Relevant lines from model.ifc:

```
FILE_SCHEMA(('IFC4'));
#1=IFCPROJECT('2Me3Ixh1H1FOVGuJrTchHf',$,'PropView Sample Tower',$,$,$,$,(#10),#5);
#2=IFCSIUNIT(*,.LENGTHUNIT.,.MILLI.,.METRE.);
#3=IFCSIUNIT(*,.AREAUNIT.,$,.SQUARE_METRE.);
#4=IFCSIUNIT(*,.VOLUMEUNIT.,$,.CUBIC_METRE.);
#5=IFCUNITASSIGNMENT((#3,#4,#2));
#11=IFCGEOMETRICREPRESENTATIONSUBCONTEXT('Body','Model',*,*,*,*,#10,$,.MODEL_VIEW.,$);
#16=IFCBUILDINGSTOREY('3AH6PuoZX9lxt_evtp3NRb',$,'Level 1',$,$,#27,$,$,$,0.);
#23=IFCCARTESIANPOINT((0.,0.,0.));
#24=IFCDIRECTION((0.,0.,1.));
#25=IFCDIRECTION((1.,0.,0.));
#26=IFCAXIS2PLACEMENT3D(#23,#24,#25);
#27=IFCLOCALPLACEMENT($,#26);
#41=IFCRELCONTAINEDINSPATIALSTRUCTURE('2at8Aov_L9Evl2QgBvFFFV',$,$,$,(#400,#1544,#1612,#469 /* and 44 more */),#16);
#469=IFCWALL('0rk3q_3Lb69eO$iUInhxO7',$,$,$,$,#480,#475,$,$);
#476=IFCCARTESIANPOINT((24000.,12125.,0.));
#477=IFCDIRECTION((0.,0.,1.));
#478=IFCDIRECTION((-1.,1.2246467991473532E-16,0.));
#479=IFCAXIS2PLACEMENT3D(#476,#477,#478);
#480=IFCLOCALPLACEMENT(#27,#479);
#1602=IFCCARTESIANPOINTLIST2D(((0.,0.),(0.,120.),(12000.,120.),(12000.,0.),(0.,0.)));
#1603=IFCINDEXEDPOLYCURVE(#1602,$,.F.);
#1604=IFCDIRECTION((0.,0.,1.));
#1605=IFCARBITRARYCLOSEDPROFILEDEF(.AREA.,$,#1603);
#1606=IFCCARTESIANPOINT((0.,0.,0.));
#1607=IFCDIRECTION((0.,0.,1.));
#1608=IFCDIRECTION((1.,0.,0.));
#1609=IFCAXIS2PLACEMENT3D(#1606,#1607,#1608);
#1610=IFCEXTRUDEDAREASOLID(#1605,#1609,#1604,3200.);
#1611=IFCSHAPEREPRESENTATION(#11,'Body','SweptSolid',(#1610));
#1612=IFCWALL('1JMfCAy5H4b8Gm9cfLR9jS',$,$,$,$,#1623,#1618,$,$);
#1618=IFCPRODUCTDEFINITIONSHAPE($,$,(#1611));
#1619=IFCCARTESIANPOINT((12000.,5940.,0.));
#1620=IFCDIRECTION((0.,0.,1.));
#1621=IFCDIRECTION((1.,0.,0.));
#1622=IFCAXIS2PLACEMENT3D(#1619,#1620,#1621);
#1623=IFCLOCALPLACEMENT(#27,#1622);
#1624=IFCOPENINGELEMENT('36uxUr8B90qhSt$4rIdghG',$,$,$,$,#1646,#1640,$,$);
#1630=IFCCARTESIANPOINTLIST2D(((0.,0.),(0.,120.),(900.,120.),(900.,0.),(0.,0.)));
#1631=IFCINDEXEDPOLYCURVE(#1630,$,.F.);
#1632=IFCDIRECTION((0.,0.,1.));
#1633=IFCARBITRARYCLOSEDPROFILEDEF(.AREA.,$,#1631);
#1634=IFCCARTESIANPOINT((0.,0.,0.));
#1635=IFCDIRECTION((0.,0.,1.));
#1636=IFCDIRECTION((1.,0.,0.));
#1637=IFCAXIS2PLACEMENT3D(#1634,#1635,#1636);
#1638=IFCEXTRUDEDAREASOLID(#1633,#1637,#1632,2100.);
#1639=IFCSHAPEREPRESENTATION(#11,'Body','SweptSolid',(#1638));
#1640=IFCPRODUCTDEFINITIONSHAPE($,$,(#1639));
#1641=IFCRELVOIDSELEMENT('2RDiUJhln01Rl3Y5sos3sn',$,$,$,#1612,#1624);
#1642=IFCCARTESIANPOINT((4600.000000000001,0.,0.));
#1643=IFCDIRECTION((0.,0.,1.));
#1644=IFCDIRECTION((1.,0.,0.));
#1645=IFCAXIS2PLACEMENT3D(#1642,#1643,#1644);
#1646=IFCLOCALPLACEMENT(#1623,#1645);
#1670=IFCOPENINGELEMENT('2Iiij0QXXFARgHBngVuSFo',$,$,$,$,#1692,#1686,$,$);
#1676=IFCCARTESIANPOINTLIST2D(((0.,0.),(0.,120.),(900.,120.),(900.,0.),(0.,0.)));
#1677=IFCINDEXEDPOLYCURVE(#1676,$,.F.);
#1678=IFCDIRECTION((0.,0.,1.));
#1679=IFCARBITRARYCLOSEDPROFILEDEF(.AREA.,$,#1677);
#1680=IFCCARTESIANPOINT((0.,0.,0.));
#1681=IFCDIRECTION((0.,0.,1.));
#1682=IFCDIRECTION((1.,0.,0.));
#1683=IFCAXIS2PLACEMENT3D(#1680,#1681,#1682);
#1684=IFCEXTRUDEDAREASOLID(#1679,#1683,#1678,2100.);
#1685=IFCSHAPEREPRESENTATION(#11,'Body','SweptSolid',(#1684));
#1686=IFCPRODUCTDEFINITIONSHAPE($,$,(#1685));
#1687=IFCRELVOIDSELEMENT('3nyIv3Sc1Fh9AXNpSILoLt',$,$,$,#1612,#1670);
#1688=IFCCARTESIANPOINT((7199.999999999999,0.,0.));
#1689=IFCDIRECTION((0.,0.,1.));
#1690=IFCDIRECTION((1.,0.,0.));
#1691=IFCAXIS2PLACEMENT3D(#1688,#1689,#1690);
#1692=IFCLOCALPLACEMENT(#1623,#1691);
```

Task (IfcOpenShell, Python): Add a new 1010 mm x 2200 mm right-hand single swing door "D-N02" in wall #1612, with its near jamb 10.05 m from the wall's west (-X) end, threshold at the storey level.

```python
import numpy as np
import ifcopenshell
import ifcopenshell.api.feature
import ifcopenshell.api.geometry
import ifcopenshell.api.root
import ifcopenshell.api.spatial
import ifcopenshell.geom
import ifcopenshell.util.element
import ifcopenshell.util.placement
import ifcopenshell.util.representation
import ifcopenshell.util.shape
import ifcopenshell.util.unit

model = ifcopenshell.open("model.ifc")
unit_scale = ifcopenshell.util.unit.calculate_unit_scale(model)
settings = ifcopenshell.geom.settings()


def volume(element):
    """Net volume in cubic metres, openings subtracted."""
    shape = ifcopenshell.geom.create_shape(settings, element)
    return ifcopenshell.util.shape.get_volume(shape.geometry)


wall = model.by_guid("1JMfCAy5H4b8Gm9cfLR9jS")
storey = ifcopenshell.util.element.get_container(wall, ifc_class="IfcBuildingStorey")
context = ifcopenshell.util.representation.get_context(model, "Model", "Body", "MODEL_VIEW")
before = volume(wall)

width, height, from_end, sill = 1.01, 2.2, 10.05, 0.0  # metres

# The wall runs along its own X axis, and the end named is its -X end.
wall_shape = ifcopenshell.geom.create_shape(settings, wall)
x, y, z = ifcopenshell.util.shape.get_vertices(wall_shape.geometry).T
start = x.min() + from_end
face, thickness = float(y.min()), float(y.max() - y.min())
wall_matrix = ifcopenshell.util.placement.get_local_placement(wall.ObjectPlacement)
level = ifcopenshell.util.placement.get_local_placement(storey.ObjectPlacement)[2, 3]


def in_wall(x, y):
    """Placement at x, y metres in the wall's axes, at sill height."""
    matrix = wall_matrix.copy()
    matrix[:, 3] = wall_matrix @ np.array([x / unit_scale, y / unit_scale, 0.0, 1.0])
    matrix[2, 3] = level + sill / unit_scale
    return matrix


# Opening: a box that overshoots both wall faces by 50 mm.
opening = ifcopenshell.api.root.create_entity(model, ifc_class="IfcOpeningElement", predefined_type="OPENING")
box = ifcopenshell.api.geometry.add_wall_representation(
    model, context=context, length=width, height=height, thickness=thickness + 0.1
)
ifcopenshell.api.geometry.assign_representation(model, product=opening, representation=box)
ifcopenshell.api.geometry.edit_object_placement(model, product=opening, matrix=in_wall(start, face - 0.05), is_si=False)
ifcopenshell.api.feature.add_feature(model, feature=opening, element=wall)

door = ifcopenshell.api.root.create_entity(model, ifc_class="IfcDoor", name="D-N02", predefined_type="DOOR")
door.OverallWidth, door.OverallHeight = width / unit_scale, height / unit_scale
door.OperationType = "SINGLE_SWING_RIGHT"
body = ifcopenshell.api.geometry.add_door_representation(
    model,
    context=context,
    overall_width=door.OverallWidth,
    overall_height=door.OverallHeight,
    operation_type="SINGLE_SWING_RIGHT",
    lining_properties={"LiningDepth": thickness / unit_scale, "ThresholdDepth": thickness / unit_scale},
)
ifcopenshell.api.geometry.assign_representation(model, product=door, representation=body)
ifcopenshell.api.spatial.assign_container(model, products=[door], relating_structure=storey)
ifcopenshell.api.feature.add_filling(model, opening=opening, element=door)

# The lining spans the wall, so the door starts at the wall face.
ifcopenshell.api.geometry.edit_object_placement(model, product=door, matrix=in_wall(start, face), is_si=False)

after = volume(wall)

print(f"wall volume {before:.3f} -> {after:.3f} m3")

model.write("model_edited.ifc")
```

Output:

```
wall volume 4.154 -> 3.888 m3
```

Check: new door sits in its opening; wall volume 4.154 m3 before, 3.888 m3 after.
